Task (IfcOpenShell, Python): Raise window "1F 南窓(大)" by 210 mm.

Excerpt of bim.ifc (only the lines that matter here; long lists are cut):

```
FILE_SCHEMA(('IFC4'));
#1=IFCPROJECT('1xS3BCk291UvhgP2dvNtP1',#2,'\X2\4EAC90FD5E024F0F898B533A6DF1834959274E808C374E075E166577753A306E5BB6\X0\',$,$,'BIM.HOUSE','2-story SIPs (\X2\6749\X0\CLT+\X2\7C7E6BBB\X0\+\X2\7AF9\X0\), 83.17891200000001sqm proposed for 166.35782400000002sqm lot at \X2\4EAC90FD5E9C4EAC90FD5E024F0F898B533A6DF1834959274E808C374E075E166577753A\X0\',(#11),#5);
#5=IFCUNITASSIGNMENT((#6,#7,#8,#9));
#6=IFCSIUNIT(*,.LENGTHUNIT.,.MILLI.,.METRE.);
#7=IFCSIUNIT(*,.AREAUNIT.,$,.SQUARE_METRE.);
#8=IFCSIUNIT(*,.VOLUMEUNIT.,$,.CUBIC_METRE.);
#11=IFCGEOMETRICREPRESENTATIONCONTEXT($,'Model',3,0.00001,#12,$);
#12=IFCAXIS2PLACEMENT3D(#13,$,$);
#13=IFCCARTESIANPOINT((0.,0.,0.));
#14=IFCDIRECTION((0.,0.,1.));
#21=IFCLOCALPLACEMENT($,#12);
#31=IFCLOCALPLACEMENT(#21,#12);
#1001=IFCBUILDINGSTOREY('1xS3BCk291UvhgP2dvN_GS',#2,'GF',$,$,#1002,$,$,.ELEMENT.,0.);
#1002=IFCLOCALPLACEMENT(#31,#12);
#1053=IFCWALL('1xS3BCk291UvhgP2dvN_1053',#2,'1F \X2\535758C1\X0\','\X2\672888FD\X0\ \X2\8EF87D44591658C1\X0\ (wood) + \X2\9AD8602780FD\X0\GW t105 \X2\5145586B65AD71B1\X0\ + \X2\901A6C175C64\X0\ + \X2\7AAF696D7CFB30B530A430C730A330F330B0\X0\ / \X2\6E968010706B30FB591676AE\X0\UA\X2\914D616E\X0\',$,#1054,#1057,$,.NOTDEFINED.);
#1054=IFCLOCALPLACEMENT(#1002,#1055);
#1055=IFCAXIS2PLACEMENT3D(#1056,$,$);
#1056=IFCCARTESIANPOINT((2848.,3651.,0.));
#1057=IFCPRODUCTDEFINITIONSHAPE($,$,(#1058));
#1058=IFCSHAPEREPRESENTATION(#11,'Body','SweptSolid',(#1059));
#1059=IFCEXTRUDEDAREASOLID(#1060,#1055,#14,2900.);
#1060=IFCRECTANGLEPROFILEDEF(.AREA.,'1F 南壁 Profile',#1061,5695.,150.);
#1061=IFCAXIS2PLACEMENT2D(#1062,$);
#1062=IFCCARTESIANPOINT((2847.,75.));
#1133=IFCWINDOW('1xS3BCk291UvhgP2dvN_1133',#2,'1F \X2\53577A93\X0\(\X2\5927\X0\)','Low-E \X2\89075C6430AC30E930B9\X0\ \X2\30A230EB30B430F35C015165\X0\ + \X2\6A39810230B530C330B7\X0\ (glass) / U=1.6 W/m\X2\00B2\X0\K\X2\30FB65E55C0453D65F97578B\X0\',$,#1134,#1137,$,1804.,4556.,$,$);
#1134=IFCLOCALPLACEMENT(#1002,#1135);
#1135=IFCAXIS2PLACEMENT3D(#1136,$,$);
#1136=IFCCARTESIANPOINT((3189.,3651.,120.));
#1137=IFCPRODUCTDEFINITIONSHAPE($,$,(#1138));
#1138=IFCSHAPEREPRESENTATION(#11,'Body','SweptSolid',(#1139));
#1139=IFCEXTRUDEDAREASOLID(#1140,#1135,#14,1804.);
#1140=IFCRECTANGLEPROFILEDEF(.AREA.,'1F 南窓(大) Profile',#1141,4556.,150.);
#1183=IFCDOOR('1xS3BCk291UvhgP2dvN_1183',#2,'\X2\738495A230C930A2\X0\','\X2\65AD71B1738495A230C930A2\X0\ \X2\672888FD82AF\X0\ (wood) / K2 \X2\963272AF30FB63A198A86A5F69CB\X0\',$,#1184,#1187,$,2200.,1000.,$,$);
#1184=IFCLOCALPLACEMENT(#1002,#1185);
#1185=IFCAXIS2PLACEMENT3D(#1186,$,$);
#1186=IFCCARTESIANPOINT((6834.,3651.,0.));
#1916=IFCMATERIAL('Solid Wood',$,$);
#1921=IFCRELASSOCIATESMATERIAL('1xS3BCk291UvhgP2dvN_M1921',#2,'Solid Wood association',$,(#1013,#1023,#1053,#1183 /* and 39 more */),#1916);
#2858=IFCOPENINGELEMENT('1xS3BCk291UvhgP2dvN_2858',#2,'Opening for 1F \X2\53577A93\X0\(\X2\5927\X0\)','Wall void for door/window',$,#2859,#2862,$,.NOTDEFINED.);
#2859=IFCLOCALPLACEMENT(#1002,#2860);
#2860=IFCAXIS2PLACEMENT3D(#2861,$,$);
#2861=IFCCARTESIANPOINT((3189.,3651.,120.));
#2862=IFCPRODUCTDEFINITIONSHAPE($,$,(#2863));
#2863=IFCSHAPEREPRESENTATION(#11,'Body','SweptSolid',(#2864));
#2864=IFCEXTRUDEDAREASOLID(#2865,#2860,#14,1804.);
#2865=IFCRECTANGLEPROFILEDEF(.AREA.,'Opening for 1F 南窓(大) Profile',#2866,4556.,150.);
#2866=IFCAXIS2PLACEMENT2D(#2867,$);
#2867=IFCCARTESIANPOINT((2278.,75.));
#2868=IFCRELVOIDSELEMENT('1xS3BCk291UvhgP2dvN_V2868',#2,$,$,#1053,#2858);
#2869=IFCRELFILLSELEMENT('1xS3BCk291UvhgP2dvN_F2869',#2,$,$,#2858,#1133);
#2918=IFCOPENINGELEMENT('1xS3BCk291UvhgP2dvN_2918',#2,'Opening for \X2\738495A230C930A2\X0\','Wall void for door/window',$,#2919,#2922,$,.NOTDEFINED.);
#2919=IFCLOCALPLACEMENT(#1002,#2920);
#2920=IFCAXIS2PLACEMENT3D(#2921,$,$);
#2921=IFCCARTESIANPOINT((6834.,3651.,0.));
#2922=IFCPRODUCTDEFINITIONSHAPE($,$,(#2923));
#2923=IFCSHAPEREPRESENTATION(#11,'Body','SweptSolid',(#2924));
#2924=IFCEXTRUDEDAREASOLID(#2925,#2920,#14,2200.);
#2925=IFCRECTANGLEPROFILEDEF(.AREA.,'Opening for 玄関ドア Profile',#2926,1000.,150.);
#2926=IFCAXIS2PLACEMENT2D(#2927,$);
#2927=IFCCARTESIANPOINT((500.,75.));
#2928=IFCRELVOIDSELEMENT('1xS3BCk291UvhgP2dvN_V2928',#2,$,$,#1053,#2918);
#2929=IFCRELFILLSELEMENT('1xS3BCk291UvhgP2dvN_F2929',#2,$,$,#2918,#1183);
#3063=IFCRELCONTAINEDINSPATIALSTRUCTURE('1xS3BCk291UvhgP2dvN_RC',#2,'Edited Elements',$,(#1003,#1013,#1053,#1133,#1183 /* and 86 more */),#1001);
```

```python
import numpy as np
import ifcopenshell
import ifcopenshell.api.geometry
import ifcopenshell.util.placement
import ifcopenshell.util.unit

model = ifcopenshell.open("bim.ifc")
unit_scale = ifcopenshell.util.unit.calculate_unit_scale(model)

window = model.by_id(1133)
opening = window.FillsVoids[0].RelatingOpeningElement
dz = 0.21 / unit_scale

shift = np.array([0.0, 0.0, dz])
# The window is not placed relative to its opening, so move both.
for product in (opening, window):
    matrix = ifcopenshell.util.placement.get_local_placement(product.ObjectPlacement)
    matrix[:3, 3] += shift
    ifcopenshell.api.geometry.edit_object_placement(model, product=product, matrix=matrix, is_si=False)

print(f"moved by {dz * unit_scale:+.3f} m")

model.write("bim_edited.ifc")
```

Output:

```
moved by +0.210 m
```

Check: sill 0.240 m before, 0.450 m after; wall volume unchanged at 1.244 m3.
